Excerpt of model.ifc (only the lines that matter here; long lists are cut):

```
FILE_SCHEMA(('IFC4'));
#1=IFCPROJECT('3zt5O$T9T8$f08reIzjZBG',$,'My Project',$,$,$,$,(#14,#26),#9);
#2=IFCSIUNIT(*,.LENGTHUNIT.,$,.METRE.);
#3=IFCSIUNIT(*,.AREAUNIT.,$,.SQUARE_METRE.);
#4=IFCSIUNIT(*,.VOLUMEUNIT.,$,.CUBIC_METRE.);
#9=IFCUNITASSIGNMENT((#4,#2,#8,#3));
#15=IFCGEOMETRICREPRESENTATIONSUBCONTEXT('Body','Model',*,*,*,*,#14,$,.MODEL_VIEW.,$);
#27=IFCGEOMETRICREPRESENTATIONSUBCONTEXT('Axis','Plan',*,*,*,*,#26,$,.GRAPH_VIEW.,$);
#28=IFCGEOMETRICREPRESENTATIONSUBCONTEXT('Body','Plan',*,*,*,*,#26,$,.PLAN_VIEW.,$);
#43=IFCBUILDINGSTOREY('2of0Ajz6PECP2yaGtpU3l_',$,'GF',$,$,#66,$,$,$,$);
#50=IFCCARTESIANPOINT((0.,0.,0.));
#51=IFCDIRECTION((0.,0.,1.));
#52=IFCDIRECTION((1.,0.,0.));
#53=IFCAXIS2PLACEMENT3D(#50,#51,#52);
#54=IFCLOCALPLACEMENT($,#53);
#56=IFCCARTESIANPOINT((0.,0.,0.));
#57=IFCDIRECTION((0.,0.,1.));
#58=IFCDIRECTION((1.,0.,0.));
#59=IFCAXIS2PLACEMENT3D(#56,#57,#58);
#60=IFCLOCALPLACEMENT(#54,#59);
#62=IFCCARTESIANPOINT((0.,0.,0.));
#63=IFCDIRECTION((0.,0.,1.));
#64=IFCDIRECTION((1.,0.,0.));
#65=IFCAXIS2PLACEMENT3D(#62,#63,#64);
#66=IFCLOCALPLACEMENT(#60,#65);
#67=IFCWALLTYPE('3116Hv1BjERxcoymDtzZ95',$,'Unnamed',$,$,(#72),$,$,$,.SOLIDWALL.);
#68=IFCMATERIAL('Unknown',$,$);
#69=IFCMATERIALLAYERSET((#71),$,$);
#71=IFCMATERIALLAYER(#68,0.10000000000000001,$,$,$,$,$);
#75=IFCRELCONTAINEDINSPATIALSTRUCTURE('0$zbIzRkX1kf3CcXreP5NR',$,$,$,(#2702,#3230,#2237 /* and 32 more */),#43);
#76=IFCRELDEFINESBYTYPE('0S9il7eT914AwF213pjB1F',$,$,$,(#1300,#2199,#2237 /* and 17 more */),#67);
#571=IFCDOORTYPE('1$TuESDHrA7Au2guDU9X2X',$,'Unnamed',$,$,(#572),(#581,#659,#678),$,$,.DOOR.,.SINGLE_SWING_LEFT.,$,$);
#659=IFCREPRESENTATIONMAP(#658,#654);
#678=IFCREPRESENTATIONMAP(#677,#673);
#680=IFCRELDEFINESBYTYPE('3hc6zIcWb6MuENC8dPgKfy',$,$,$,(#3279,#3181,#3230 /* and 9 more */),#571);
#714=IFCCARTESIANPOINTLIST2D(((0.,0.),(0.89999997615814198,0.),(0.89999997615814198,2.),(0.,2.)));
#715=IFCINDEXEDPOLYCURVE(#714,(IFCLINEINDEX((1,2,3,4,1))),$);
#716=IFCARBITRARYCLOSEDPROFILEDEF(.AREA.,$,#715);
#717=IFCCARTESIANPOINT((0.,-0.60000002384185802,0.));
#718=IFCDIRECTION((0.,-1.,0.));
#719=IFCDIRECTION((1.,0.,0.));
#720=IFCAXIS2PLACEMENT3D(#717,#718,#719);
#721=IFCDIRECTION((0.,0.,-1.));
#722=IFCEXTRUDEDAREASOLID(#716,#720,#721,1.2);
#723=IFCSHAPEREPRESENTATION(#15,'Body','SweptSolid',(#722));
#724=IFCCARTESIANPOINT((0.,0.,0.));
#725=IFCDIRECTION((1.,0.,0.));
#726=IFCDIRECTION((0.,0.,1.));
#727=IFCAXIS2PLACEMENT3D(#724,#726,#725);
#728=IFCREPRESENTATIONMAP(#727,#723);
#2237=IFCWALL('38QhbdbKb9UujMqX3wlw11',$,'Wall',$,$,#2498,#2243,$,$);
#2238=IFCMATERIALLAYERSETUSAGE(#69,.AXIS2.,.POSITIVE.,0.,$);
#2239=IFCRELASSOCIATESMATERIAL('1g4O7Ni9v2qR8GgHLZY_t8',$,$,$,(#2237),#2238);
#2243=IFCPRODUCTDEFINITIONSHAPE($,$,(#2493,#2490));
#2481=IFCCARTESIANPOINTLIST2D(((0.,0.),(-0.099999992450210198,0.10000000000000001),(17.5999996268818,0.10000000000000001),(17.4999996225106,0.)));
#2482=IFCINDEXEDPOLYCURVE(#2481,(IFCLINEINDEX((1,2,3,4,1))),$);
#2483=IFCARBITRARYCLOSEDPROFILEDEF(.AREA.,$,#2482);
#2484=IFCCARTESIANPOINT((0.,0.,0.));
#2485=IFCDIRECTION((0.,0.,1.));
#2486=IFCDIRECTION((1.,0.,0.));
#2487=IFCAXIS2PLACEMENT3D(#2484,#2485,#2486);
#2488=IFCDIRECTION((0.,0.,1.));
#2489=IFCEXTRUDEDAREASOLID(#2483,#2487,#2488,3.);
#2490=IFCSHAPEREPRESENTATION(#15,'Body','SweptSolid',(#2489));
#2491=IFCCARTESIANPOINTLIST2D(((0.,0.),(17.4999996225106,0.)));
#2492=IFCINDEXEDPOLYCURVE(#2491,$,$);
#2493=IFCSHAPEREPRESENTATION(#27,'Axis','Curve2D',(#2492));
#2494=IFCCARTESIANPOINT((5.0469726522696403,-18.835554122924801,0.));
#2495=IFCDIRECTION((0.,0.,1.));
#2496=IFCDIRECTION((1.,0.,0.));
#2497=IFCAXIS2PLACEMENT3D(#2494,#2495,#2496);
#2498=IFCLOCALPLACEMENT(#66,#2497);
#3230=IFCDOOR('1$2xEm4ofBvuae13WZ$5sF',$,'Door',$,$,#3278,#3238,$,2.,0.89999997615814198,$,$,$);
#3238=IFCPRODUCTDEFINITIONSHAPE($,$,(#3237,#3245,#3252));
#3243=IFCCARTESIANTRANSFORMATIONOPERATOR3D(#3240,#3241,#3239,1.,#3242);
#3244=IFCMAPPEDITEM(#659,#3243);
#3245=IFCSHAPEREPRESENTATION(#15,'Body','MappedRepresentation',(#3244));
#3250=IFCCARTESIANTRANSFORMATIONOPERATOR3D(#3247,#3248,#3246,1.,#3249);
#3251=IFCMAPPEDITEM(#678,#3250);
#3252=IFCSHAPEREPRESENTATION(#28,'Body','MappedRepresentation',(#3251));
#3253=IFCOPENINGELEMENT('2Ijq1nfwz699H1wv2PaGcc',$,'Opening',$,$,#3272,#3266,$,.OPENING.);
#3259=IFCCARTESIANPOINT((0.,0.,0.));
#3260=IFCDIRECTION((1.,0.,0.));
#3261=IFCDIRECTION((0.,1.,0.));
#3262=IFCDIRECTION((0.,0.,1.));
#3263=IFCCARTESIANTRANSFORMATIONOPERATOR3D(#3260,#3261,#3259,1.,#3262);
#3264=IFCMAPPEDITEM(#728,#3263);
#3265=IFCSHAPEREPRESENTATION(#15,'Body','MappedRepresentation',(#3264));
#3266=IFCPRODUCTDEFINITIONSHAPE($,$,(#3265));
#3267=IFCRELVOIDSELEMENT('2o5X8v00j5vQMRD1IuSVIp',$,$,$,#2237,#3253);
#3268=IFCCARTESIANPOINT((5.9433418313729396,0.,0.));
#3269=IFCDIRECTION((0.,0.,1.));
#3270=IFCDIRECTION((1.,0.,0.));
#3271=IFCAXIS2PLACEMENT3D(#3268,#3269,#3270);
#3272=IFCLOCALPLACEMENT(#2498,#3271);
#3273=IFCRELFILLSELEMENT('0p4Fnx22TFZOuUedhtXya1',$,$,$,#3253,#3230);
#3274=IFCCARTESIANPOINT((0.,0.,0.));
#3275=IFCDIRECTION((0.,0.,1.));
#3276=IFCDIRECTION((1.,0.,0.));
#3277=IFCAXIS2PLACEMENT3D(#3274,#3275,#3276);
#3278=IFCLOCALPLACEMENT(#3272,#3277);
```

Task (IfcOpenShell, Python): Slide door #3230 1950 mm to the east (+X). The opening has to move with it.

```python
import ifcopenshell
import ifcopenshell.api.geometry
import ifcopenshell.util.placement
import ifcopenshell.util.unit

model = ifcopenshell.open("model.ifc")
unit_scale = ifcopenshell.util.unit.calculate_unit_scale(model)

door = model.by_guid("1$2xEm4ofBvuae13WZ$5sF")
opening = door.FillsVoids[0].RelatingOpeningElement
wall = opening.VoidsElements[0].RelatingBuildingElement

wall_matrix = ifcopenshell.util.placement.get_local_placement(wall.ObjectPlacement)
shift = wall_matrix[:3, 0] * 1.95 / unit_scale
before = ifcopenshell.util.placement.get_local_placement(door.ObjectPlacement)[:3, 3].copy()

# The door is placed relative to its opening, so it follows when the opening moves.
matrix = ifcopenshell.util.placement.get_local_placement(opening.ObjectPlacement)
matrix[:3, 3] += shift
ifcopenshell.api.geometry.edit_object_placement(
    model, product=opening, matrix=matrix, is_si=False, should_transform_children=True
)

after = ifcopenshell.util.placement.get_local_placement(door.ObjectPlacement)[:3, 3]
print("door moved by", (after - before).round(3) + 0.0)

model.write("model_rev.ifc")
```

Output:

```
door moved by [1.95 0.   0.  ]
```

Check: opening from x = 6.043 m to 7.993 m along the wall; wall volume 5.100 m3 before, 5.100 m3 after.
